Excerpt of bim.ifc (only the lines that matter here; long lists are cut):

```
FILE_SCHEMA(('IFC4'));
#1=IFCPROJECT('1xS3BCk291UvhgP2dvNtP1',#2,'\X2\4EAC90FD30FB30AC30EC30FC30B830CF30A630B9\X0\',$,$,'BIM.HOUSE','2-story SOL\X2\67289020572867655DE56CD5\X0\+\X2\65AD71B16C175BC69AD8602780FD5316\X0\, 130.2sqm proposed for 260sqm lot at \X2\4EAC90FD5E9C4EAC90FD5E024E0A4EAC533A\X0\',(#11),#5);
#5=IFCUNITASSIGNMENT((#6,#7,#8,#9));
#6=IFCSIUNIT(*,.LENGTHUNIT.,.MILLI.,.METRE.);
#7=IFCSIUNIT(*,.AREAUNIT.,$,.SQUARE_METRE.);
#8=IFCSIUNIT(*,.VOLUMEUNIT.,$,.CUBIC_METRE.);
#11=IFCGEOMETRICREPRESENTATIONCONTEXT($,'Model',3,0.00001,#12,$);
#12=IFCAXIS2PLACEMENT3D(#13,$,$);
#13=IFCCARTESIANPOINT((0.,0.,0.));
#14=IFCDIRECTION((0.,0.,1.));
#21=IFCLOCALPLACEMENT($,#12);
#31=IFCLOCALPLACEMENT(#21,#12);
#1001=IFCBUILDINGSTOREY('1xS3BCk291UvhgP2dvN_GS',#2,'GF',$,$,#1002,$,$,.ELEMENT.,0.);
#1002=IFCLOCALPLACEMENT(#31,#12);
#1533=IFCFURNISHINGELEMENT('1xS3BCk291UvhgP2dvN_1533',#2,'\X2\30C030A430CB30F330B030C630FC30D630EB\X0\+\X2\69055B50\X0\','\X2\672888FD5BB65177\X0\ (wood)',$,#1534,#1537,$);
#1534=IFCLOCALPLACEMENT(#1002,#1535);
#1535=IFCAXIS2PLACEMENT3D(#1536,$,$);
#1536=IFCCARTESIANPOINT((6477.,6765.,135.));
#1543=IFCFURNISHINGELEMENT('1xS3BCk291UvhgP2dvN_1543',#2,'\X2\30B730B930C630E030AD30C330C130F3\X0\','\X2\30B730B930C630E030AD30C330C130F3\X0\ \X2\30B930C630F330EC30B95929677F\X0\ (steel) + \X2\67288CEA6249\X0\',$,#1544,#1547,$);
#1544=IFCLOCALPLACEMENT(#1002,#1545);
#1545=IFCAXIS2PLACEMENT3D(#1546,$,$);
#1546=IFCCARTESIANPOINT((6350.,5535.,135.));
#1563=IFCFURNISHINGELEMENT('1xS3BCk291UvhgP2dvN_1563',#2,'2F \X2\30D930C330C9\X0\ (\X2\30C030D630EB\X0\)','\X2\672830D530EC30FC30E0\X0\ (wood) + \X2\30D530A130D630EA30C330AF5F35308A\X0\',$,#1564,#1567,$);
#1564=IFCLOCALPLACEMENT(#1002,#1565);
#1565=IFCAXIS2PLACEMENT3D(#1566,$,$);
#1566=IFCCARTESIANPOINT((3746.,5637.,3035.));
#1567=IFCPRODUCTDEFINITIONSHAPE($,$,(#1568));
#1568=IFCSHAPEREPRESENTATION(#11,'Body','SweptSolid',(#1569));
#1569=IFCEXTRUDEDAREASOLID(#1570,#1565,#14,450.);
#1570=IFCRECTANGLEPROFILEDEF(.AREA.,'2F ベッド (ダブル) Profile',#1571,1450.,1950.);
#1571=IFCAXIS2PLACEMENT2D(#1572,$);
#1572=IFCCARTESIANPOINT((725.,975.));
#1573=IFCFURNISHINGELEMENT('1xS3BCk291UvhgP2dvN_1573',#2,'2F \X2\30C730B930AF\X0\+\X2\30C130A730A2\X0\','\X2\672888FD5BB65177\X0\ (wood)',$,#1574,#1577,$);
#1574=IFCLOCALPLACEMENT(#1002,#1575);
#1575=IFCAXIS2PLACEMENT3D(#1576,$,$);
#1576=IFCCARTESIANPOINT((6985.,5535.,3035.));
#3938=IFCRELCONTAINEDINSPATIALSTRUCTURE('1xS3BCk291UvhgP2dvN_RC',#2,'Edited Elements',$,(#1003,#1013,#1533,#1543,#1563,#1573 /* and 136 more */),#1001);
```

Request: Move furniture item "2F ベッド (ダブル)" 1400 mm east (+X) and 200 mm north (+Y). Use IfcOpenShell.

```python
import ifcopenshell
import ifcopenshell.api.geometry
import ifcopenshell.util.placement

model = ifcopenshell.open("bim.ifc")

item = model.by_guid("1xS3BCk291UvhgP2dvN_1563")
matrix = ifcopenshell.util.placement.get_local_placement(item.ObjectPlacement)
matrix[0, 3] += 1400.0
matrix[1, 3] += 200.0
ifcopenshell.api.geometry.edit_object_placement(model, product=item, matrix=matrix, is_si=False)

print(ifcopenshell.util.placement.get_local_placement(item.ObjectPlacement).round(3) + 0.0)

model.write("bim_edited.ifc")
```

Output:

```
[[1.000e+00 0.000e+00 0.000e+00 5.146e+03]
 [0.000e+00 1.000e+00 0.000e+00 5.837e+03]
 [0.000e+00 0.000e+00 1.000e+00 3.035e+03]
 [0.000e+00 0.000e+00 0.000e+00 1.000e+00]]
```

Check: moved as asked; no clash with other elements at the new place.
